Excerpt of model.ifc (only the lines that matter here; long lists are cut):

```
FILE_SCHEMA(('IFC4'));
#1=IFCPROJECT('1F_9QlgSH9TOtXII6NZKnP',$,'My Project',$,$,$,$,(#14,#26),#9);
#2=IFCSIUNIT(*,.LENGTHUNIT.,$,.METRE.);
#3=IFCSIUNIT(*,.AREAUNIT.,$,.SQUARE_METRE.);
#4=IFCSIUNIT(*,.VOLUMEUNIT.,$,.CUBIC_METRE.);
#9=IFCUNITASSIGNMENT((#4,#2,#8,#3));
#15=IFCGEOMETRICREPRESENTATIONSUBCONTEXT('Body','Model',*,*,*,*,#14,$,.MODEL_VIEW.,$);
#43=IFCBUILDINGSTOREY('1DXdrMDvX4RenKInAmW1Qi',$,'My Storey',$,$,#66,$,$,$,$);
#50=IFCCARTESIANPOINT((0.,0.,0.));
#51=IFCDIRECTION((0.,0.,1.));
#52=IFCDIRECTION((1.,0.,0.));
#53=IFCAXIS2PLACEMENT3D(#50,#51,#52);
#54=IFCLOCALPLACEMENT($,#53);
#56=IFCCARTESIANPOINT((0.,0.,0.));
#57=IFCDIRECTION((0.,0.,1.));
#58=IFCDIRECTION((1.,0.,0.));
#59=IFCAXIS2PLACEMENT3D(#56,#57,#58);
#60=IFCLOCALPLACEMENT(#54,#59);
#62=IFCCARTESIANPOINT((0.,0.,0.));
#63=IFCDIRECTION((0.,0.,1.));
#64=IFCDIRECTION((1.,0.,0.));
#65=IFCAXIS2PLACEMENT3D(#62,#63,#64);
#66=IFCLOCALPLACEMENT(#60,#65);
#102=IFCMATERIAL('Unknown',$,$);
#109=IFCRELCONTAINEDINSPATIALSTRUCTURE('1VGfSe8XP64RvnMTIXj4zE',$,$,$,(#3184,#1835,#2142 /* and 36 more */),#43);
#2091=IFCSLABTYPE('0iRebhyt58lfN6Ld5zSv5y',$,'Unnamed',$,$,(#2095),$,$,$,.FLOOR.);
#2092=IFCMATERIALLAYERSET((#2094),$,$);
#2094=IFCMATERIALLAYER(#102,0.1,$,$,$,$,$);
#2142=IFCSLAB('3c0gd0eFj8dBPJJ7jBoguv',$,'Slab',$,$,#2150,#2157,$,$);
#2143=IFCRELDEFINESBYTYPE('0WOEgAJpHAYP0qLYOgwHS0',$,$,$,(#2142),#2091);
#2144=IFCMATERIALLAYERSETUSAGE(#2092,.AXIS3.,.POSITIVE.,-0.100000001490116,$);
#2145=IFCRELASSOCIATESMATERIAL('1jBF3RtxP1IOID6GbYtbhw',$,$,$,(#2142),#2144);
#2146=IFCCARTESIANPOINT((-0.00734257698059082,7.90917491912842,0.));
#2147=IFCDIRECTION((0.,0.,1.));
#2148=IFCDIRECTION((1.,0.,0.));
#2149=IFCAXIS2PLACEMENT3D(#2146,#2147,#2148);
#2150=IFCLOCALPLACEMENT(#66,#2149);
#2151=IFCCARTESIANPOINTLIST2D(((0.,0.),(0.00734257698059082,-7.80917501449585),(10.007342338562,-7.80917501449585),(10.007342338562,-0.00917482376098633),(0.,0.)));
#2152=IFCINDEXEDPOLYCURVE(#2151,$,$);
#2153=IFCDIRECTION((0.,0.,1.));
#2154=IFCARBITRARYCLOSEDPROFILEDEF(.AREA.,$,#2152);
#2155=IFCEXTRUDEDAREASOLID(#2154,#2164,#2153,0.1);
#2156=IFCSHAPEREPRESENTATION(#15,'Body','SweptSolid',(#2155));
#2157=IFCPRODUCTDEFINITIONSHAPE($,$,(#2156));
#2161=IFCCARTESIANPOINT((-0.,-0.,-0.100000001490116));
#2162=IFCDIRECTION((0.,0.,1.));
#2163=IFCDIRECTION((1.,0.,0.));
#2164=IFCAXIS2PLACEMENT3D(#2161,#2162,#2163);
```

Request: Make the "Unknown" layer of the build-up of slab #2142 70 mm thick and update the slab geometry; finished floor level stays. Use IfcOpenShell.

```python
import ifcopenshell
import ifcopenshell.util.element
import ifcopenshell.util.representation

model = ifcopenshell.open("model.ifc")

layer_set = model.by_id(2092)
layer = next(l for l in layer_set.MaterialLayers if l.Material and l.Material.Name == "Unknown")
change = 0.07 - layer.LayerThickness
layer.LayerThickness += change

# Geometry does not follow the layer set by itself.
slabs = [e for e in ifcopenshell.util.element.get_elements_by_material(model, layer_set) if e.is_a("IfcSlab")]
for slab in sorted(slabs, key=lambda e: e.id()):
    body = ifcopenshell.util.representation.get_representation(slab, "Model", "Body")
    solid = body.Items[0]
    old_depth = solid.Depth
    solid.Depth += change
    # Extruded upwards: lower the start of the extrusion so the top stays.
    x, y, z = solid.Position.Location.Coordinates
    solid.Position.Location = model.createIfcCartesianPoint((x, y, z - change))
    print(slab.id(), f"{old_depth:g} -> {solid.Depth:g}")

# The layers are counted up from the underside, which has moved.
for usage in {ifcopenshell.util.element.get_material(slab) for slab in slabs}:
    usage.OffsetFromReferenceLine -= change

model.write("model-out.ifc")
```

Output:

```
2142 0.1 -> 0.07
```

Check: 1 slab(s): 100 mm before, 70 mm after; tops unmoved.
